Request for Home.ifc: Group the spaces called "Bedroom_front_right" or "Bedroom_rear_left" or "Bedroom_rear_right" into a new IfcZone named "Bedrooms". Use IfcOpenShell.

First a look at what the model holds.

```python
import ifcopenshell

model = ifcopenshell.open("Home.ifc")
print(model.schema)
seen = {}
for space in model.by_type("IfcSpace"):
    seen[space.LongName] = seen.get(space.LongName, 0) + 1
for name, count in sorted(seen.items(), key=str):
    print(count, "x", name)
print("zones:", [z.Name for z in model.by_type("IfcZone")][:20])
```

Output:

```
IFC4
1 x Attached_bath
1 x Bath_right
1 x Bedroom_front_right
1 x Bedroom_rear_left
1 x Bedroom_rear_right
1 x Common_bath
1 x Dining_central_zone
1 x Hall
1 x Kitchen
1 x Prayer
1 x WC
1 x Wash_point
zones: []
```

```python
import ifcopenshell
import ifcopenshell.api.group
import ifcopenshell.api.root

model = ifcopenshell.open("Home.ifc")

names = {"Bedroom_front_right", "Bedroom_rear_left", "Bedroom_rear_right"}
spaces = [s for s in model.by_type("IfcSpace") if s.LongName in names]

zone = ifcopenshell.api.root.create_entity(model, ifc_class="IfcZone", name="Bedrooms")
ifcopenshell.api.group.assign_group(model, products=spaces, group=zone)
print(len(spaces), "spaces in", zone.Name)

model.write("Home-out.ifc")
```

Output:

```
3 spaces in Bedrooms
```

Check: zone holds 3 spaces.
